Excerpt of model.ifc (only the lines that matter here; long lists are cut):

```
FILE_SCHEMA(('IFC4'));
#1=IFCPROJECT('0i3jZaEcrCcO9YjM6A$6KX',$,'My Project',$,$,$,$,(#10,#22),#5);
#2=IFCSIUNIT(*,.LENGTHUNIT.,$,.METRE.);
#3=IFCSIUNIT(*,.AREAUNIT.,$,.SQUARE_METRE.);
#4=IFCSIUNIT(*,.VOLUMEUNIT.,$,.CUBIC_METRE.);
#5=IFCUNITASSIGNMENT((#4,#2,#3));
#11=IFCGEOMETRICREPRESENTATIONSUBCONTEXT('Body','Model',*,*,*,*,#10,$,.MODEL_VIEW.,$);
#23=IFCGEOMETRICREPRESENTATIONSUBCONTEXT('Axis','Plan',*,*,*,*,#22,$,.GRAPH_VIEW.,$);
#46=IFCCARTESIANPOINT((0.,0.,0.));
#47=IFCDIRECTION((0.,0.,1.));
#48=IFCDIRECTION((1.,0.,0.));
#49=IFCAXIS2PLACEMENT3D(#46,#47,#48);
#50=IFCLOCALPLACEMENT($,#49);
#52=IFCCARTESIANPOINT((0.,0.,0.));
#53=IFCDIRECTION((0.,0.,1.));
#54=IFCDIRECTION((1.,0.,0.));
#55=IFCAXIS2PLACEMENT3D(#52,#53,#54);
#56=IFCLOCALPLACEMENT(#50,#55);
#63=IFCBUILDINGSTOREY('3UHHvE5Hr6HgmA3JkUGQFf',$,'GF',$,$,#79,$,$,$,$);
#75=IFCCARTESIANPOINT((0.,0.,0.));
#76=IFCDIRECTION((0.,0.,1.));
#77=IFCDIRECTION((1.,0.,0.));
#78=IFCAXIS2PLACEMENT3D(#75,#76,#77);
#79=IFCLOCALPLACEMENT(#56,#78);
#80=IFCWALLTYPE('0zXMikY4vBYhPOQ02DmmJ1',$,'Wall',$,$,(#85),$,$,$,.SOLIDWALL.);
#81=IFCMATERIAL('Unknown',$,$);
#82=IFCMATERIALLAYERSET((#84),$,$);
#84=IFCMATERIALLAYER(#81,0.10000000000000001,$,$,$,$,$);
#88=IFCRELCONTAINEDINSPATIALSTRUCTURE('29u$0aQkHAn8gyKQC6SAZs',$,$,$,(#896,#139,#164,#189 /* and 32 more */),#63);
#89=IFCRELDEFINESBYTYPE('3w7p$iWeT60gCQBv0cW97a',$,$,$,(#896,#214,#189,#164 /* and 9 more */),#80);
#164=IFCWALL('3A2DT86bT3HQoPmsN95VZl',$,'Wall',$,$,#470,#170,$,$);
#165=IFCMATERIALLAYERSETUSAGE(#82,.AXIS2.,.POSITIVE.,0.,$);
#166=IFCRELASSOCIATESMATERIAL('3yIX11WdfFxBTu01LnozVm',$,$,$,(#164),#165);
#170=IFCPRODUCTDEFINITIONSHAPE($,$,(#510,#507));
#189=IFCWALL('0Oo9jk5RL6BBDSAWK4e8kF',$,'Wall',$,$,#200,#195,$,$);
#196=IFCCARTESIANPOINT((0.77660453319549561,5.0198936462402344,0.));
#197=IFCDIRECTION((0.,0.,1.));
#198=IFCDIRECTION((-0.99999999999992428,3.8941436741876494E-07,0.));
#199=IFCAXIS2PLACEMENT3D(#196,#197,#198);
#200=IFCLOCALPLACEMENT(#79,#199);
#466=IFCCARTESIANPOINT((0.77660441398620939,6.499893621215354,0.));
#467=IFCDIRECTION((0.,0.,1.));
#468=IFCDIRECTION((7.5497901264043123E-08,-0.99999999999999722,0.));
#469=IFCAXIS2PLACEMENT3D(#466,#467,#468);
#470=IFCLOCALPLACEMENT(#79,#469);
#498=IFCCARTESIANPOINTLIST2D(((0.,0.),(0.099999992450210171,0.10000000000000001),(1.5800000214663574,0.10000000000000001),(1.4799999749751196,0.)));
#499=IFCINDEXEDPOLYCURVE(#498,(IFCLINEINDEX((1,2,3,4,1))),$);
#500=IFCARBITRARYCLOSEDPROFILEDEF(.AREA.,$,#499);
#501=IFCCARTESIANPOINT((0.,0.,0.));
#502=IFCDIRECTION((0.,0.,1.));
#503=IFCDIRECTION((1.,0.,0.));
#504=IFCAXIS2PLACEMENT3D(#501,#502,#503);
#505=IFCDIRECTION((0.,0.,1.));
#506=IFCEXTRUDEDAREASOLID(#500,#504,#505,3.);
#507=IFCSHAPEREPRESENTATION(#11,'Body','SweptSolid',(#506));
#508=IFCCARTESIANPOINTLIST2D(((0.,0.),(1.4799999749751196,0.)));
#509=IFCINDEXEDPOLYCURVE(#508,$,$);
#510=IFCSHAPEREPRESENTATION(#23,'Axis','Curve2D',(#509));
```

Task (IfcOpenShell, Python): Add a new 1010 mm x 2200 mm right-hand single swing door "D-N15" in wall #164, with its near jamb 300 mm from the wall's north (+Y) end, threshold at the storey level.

```python
import numpy as np
import ifcopenshell
import ifcopenshell.api.feature
import ifcopenshell.api.geometry
import ifcopenshell.api.root
import ifcopenshell.api.spatial
import ifcopenshell.geom
import ifcopenshell.util.element
import ifcopenshell.util.placement
import ifcopenshell.util.representation
import ifcopenshell.util.shape
import ifcopenshell.util.unit

model = ifcopenshell.open("model.ifc")
unit_scale = ifcopenshell.util.unit.calculate_unit_scale(model)
settings = ifcopenshell.geom.settings()


def volume(element):
    """Net volume in cubic metres, openings subtracted."""
    shape = ifcopenshell.geom.create_shape(settings, element)
    return ifcopenshell.util.shape.get_volume(shape.geometry)


wall = model.by_guid("3A2DT86bT3HQoPmsN95VZl")
storey = ifcopenshell.util.element.get_container(wall, ifc_class="IfcBuildingStorey")
context = ifcopenshell.util.representation.get_context(model, "Model", "Body", "MODEL_VIEW")
before = volume(wall)

width, height, from_end, sill = 1.01, 2.2, 0.3, 0.0  # metres

# The wall runs along its own X axis, and the end named is its -X end.
wall_shape = ifcopenshell.geom.create_shape(settings, wall)
x, y, z = ifcopenshell.util.shape.get_vertices(wall_shape.geometry).T
start = x.min() + from_end
face, thickness = float(y.min()), float(y.max() - y.min())
wall_matrix = ifcopenshell.util.placement.get_local_placement(wall.ObjectPlacement)
level = ifcopenshell.util.placement.get_local_placement(storey.ObjectPlacement)[2, 3]


def in_wall(x, y):
    """Placement at x, y metres in the wall's axes, at sill height."""
    matrix = wall_matrix.copy()
    matrix[:, 3] = wall_matrix @ np.array([x / unit_scale, y / unit_scale, 0.0, 1.0])
    matrix[2, 3] = level + sill / unit_scale
    return matrix


# Opening: a box that overshoots both wall faces by 50 mm.
opening = ifcopenshell.api.root.create_entity(model, ifc_class="IfcOpeningElement", predefined_type="OPENING")
box = ifcopenshell.api.geometry.add_wall_representation(
    model, context=context, length=width, height=height, thickness=thickness + 0.1
)
ifcopenshell.api.geometry.assign_representation(model, product=opening, representation=box)
ifcopenshell.api.geometry.edit_object_placement(model, product=opening, matrix=in_wall(start, face - 0.05), is_si=False)
ifcopenshell.api.feature.add_feature(model, feature=opening, element=wall)

door = ifcopenshell.api.root.create_entity(model, ifc_class="IfcDoor", name="D-N15", predefined_type="DOOR")
door.OverallWidth, door.OverallHeight = width / unit_scale, height / unit_scale
door.OperationType = "SINGLE_SWING_RIGHT"
body = ifcopenshell.api.geometry.add_door_representation(
    model,
    context=context,
    overall_width=door.OverallWidth,
    overall_height=door.OverallHeight,
    operation_type="SINGLE_SWING_RIGHT",
    lining_properties={"LiningDepth": thickness / unit_scale, "ThresholdDepth": thickness / unit_scale},
)
ifcopenshell.api.geometry.assign_representation(model, product=door, representation=body)
ifcopenshell.api.spatial.assign_container(model, products=[door], relating_structure=storey)
ifcopenshell.api.feature.add_filling(model, opening=opening, element=door)

# The lining spans the wall, so the door starts at the wall face.
ifcopenshell.api.geometry.edit_object_placement(model, product=door, matrix=in_wall(start, face), is_si=False)

after = volume(wall)

print(f"wall volume {before:.3f} -> {after:.3f} m3")

model.write("model_v2.ifc")
```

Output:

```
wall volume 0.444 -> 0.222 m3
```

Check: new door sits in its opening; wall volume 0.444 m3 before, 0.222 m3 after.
